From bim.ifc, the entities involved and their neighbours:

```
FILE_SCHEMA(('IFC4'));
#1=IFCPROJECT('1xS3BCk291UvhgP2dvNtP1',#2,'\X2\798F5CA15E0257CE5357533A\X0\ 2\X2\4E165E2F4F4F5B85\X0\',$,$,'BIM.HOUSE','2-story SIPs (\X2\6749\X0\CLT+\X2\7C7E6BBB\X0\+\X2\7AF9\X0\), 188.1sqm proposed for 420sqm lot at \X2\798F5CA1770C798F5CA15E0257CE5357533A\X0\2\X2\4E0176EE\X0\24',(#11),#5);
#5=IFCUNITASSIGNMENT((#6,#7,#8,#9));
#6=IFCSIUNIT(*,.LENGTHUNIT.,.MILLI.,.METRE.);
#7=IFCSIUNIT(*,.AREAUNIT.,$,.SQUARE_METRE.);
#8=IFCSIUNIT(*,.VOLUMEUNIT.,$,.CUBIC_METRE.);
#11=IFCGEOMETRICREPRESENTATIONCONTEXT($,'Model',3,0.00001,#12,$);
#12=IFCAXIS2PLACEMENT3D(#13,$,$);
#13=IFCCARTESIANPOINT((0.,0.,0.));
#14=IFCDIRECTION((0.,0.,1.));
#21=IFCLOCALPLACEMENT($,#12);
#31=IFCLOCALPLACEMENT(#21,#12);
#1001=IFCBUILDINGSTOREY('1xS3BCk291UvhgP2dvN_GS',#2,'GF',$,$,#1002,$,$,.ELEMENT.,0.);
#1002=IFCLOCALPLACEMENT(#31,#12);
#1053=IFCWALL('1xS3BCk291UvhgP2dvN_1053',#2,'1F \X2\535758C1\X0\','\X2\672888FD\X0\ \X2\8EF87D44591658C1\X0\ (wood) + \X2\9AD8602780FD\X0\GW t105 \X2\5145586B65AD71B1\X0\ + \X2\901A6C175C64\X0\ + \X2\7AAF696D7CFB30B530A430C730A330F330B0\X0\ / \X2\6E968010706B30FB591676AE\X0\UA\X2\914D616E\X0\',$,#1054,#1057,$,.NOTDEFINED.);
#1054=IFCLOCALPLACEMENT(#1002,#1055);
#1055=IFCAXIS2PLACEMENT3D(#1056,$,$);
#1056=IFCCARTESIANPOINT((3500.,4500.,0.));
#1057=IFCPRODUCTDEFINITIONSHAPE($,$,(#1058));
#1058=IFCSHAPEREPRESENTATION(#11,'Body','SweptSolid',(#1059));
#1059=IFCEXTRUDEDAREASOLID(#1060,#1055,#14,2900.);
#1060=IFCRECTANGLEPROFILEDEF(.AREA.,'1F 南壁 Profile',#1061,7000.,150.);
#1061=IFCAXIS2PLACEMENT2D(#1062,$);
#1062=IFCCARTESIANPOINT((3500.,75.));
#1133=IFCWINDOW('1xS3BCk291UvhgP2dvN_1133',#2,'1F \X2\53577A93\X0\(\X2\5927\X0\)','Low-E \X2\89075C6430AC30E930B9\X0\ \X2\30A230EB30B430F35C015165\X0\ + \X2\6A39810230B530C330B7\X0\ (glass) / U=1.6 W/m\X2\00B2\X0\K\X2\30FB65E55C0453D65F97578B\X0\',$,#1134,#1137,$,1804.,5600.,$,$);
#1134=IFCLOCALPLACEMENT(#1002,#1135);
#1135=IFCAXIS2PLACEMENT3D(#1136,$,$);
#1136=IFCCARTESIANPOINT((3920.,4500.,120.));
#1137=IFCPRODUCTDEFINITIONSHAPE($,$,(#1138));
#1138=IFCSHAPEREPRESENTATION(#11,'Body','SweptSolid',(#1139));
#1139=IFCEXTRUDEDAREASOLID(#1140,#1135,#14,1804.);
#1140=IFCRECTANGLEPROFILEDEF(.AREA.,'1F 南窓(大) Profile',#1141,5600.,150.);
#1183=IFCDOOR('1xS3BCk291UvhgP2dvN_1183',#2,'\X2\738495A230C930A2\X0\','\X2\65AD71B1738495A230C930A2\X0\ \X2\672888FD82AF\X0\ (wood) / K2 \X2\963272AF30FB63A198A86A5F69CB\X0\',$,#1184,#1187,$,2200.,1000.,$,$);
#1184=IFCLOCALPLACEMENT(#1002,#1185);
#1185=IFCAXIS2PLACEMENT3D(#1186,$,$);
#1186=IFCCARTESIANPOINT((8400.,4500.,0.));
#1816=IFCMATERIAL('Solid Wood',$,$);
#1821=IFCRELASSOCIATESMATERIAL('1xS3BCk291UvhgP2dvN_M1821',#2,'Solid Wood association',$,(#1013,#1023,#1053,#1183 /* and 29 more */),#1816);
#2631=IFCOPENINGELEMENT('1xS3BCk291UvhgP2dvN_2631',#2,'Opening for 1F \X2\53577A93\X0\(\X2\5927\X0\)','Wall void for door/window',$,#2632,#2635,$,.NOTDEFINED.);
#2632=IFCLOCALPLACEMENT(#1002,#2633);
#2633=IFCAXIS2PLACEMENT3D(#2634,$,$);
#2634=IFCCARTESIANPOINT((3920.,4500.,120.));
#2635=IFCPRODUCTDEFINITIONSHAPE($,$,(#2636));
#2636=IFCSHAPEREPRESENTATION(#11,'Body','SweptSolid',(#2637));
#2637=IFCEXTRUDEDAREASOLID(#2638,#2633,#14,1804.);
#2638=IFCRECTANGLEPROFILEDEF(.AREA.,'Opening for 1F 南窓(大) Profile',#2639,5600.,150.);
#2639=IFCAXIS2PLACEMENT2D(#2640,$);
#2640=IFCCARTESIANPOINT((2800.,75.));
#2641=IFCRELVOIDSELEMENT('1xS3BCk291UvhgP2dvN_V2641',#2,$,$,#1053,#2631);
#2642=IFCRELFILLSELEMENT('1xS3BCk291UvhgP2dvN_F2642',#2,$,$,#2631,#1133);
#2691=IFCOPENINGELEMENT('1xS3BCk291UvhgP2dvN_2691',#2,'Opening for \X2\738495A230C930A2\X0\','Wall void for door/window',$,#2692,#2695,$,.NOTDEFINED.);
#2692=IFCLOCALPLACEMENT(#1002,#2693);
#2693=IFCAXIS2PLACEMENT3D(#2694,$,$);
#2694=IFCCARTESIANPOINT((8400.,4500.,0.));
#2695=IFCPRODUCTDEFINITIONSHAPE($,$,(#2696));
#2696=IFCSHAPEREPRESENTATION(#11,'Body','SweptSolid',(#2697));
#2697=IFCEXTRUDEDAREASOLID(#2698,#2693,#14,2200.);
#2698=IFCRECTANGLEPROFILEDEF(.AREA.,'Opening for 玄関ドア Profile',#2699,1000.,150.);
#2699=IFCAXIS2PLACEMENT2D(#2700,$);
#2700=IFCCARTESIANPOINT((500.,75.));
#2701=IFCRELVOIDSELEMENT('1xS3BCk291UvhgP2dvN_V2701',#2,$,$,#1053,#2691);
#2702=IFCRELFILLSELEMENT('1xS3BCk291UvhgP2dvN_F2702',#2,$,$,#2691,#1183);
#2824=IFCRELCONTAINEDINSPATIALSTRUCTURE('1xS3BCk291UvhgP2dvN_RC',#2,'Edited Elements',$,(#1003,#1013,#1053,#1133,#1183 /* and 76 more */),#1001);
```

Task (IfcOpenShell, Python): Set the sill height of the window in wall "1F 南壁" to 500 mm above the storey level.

```python
import numpy as np
import ifcopenshell
import ifcopenshell.api.geometry
import ifcopenshell.geom
import ifcopenshell.util.element
import ifcopenshell.util.placement
import ifcopenshell.util.shape
import ifcopenshell.util.unit

model = ifcopenshell.open("bim.ifc")
unit_scale = ifcopenshell.util.unit.calculate_unit_scale(model)

window = model.by_guid("1xS3BCk291UvhgP2dvN_1133")
opening = window.FillsVoids[0].RelatingOpeningElement
storey = ifcopenshell.util.element.get_container(window, ifc_class="IfcBuildingStorey")
level = ifcopenshell.util.placement.get_local_placement(storey.ObjectPlacement)[2, 3]

# The opening's origin need not be at the sill, so measure its lowest point.
shape = ifcopenshell.geom.create_shape(ifcopenshell.geom.settings(), opening)
bottom = ifcopenshell.util.shape.get_shape_bottom_elevation(shape, shape.geometry) / unit_scale
dz = level + 0.5 / unit_scale - bottom

shift = np.array([0.0, 0.0, dz])
# The window is not placed relative to its opening, so move both.
for product in (opening, window):
    matrix = ifcopenshell.util.placement.get_local_placement(product.ObjectPlacement)
    matrix[:3, 3] += shift
    ifcopenshell.api.geometry.edit_object_placement(model, product=product, matrix=matrix, is_si=False)

print(f"moved by {dz * unit_scale:+.3f} m")

model.write("bim_updated.ifc")
```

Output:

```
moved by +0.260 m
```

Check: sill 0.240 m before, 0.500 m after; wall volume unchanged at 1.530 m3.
